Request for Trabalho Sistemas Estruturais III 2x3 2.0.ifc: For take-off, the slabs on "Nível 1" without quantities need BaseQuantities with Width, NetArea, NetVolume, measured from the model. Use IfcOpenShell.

First a look at what the model holds.

```python
import ifcopenshell
import ifcopenshell.util.element
import ifcopenshell.util.unit

model = ifcopenshell.open("Trabalho Sistemas Estruturais III 2x3 2.0.ifc")
print(model.schema)
for unit_type in ("LENGTHUNIT", "AREAUNIT", "VOLUMEUNIT"):
    print(unit_type, ifcopenshell.util.unit.calculate_unit_scale(model, unit_type))
storey = next(s for s in model.by_type("IfcBuildingStorey") if s.Name == "Nível 1")
slabs = [e for e in ifcopenshell.util.element.get_decomposition(storey) if e.is_a("IfcSlab")]
for e in sorted(slabs, key=lambda e: e.id()):
    print(e.id(), e.is_a(), e.Name, list(ifcopenshell.util.element.get_psets(e, qtos_only=True)), sep=" | ")
```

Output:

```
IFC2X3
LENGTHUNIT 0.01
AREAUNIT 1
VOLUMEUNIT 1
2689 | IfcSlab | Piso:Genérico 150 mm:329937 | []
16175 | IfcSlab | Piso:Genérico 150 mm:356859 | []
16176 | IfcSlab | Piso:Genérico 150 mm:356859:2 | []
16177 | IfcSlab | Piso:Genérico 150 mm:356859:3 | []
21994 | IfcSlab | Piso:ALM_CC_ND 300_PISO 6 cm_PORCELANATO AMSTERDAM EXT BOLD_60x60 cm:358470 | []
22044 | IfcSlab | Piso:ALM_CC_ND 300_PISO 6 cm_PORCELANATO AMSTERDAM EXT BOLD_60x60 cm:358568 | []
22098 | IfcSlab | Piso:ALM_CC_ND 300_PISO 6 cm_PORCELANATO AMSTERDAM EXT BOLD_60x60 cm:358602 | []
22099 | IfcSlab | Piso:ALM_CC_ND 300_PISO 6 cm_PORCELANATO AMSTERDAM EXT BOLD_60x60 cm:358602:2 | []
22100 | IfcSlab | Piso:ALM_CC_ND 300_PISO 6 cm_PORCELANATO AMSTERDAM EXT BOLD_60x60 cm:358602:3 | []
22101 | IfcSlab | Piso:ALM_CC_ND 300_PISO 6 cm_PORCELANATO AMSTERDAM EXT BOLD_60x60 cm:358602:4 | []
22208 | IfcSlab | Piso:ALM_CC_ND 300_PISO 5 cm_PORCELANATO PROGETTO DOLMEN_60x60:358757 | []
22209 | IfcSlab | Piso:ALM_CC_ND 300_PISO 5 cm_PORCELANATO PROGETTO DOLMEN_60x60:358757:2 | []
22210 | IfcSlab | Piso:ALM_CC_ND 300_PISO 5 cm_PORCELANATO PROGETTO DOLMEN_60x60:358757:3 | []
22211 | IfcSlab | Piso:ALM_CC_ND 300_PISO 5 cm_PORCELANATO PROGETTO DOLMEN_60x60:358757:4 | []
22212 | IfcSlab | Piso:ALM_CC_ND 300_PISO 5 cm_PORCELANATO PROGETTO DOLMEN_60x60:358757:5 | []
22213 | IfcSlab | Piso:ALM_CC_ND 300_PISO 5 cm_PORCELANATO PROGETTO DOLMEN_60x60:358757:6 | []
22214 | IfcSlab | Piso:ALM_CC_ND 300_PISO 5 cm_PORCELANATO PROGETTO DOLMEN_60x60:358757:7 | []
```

```python
import ifcopenshell
import ifcopenshell.api.pset
import ifcopenshell.geom
import ifcopenshell.util.element
import ifcopenshell.util.shape
import ifcopenshell.util.unit

model = ifcopenshell.open("Trabalho Sistemas Estruturais III 2x3 2.0.ifc")
unit_scale = ifcopenshell.util.unit.calculate_unit_scale(model)
area_scale = ifcopenshell.util.unit.calculate_unit_scale(model, "AREAUNIT")
volume_scale = ifcopenshell.util.unit.calculate_unit_scale(model, "VOLUMEUNIT")
settings = ifcopenshell.geom.settings()

storey = next(s for s in model.by_type("IfcBuildingStorey") if s.Name == "Nível 1")
slabs = [e for e in ifcopenshell.util.element.get_decomposition(storey) if e.is_a("IfcSlab")]

for e in sorted(slabs, key=lambda e: e.id()):
    if ifcopenshell.util.element.get_psets(e, qtos_only=True, should_inherit=False):
        continue
    # Geometry comes back in metres, in the element's own axes.
    shape = ifcopenshell.geom.create_shape(settings, e)
    values = {
        "Width": ifcopenshell.util.shape.get_z(shape.geometry) / unit_scale,
        "NetArea": ifcopenshell.util.shape.get_footprint_area(shape.geometry) / area_scale,
        "NetVolume": ifcopenshell.util.shape.get_volume(shape.geometry) / volume_scale,
    }
    qto = ifcopenshell.api.pset.add_qto(model, product=e, name="BaseQuantities")
    ifcopenshell.api.pset.edit_qto(model, qto=qto, properties=values)
    print(e.id(), {k: round(v, 3) for k, v in values.items()})

model.write("Trabalho Sistemas Estruturais III 2x3 2.0-out.ifc")
```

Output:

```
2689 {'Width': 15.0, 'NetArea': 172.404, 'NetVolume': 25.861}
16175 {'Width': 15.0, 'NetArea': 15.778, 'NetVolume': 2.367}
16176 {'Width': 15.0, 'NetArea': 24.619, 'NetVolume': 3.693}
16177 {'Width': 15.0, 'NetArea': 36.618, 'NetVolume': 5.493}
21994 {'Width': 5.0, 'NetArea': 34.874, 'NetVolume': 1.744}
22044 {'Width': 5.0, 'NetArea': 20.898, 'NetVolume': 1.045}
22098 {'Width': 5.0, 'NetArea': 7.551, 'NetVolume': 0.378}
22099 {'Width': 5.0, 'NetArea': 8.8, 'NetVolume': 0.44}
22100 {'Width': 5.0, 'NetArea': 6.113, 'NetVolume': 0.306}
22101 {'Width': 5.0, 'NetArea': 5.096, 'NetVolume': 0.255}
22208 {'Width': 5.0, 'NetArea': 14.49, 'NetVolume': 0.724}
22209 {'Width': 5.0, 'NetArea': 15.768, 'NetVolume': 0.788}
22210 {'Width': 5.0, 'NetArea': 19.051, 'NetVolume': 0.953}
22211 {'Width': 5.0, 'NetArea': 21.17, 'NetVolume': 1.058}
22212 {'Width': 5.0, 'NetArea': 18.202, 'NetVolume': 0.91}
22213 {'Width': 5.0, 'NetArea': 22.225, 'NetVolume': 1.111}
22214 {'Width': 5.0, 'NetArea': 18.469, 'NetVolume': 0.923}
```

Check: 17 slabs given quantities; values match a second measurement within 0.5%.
